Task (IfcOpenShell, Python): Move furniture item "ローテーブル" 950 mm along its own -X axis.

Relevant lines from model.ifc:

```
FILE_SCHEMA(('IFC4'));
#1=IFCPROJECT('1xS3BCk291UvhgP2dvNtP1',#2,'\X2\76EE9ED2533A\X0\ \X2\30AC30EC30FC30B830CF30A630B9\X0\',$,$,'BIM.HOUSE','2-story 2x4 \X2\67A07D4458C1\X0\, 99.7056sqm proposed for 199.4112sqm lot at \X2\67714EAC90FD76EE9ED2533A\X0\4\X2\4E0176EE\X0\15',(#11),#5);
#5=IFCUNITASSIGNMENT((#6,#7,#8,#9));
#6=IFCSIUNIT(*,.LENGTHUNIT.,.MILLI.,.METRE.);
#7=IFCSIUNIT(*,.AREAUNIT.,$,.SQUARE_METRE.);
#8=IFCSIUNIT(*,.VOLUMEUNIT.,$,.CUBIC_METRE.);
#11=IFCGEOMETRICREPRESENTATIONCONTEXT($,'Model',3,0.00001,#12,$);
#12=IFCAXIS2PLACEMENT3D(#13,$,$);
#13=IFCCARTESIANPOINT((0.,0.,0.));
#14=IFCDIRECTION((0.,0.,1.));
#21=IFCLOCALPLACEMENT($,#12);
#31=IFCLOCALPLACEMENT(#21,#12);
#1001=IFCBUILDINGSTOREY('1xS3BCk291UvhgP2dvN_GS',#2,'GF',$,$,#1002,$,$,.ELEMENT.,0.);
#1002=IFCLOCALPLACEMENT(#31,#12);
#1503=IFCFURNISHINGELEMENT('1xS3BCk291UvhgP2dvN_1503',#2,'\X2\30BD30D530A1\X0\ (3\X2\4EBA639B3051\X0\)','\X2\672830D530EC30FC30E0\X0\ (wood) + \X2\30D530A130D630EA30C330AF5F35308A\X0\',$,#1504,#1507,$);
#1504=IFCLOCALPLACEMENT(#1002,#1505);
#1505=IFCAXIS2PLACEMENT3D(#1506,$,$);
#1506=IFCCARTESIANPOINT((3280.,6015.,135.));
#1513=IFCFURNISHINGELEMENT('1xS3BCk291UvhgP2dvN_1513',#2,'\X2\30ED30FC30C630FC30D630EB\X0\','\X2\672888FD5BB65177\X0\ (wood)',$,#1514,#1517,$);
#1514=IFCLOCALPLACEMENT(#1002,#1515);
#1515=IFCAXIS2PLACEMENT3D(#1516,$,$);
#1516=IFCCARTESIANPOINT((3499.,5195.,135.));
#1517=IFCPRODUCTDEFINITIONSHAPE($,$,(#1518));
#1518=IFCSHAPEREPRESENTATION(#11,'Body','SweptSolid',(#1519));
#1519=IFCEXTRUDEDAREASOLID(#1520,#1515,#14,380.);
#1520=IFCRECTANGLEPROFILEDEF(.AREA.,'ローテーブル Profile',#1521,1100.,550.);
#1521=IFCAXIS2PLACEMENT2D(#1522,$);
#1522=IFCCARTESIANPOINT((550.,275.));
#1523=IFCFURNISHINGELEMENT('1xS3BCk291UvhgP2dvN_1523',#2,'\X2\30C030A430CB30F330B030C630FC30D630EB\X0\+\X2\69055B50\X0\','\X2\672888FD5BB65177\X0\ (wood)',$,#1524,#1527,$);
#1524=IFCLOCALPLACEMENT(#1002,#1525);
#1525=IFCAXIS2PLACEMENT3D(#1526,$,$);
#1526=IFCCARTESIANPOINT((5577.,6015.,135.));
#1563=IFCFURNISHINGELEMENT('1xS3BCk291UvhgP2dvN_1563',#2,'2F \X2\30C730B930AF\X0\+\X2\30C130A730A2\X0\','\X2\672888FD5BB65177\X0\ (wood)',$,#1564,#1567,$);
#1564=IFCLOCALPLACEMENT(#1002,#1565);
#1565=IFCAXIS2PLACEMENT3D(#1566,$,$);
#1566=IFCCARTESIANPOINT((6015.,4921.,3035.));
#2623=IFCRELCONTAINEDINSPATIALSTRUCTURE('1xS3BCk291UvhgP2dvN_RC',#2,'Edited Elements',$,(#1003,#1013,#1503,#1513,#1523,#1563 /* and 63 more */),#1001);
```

```python
import ifcopenshell
import ifcopenshell.api.geometry
import ifcopenshell.util.placement
import ifcopenshell.util.unit

model = ifcopenshell.open("model.ifc")
unit_scale = ifcopenshell.util.unit.calculate_unit_scale(model)

item = model.by_guid("1xS3BCk291UvhgP2dvN_1513")
matrix = ifcopenshell.util.placement.get_local_placement(item.ObjectPlacement)
matrix[:3, 3] -= matrix[:3, 0] * 0.95 / unit_scale
ifcopenshell.api.geometry.edit_object_placement(model, product=item, matrix=matrix, is_si=False)

print(ifcopenshell.util.placement.get_local_placement(item.ObjectPlacement).round(3) + 0.0)

model.write("model_edited.ifc")
```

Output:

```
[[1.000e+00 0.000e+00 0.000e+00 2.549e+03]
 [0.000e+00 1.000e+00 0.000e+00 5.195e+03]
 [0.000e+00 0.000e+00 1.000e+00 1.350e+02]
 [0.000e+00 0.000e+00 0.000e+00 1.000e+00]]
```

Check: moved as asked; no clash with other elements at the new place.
